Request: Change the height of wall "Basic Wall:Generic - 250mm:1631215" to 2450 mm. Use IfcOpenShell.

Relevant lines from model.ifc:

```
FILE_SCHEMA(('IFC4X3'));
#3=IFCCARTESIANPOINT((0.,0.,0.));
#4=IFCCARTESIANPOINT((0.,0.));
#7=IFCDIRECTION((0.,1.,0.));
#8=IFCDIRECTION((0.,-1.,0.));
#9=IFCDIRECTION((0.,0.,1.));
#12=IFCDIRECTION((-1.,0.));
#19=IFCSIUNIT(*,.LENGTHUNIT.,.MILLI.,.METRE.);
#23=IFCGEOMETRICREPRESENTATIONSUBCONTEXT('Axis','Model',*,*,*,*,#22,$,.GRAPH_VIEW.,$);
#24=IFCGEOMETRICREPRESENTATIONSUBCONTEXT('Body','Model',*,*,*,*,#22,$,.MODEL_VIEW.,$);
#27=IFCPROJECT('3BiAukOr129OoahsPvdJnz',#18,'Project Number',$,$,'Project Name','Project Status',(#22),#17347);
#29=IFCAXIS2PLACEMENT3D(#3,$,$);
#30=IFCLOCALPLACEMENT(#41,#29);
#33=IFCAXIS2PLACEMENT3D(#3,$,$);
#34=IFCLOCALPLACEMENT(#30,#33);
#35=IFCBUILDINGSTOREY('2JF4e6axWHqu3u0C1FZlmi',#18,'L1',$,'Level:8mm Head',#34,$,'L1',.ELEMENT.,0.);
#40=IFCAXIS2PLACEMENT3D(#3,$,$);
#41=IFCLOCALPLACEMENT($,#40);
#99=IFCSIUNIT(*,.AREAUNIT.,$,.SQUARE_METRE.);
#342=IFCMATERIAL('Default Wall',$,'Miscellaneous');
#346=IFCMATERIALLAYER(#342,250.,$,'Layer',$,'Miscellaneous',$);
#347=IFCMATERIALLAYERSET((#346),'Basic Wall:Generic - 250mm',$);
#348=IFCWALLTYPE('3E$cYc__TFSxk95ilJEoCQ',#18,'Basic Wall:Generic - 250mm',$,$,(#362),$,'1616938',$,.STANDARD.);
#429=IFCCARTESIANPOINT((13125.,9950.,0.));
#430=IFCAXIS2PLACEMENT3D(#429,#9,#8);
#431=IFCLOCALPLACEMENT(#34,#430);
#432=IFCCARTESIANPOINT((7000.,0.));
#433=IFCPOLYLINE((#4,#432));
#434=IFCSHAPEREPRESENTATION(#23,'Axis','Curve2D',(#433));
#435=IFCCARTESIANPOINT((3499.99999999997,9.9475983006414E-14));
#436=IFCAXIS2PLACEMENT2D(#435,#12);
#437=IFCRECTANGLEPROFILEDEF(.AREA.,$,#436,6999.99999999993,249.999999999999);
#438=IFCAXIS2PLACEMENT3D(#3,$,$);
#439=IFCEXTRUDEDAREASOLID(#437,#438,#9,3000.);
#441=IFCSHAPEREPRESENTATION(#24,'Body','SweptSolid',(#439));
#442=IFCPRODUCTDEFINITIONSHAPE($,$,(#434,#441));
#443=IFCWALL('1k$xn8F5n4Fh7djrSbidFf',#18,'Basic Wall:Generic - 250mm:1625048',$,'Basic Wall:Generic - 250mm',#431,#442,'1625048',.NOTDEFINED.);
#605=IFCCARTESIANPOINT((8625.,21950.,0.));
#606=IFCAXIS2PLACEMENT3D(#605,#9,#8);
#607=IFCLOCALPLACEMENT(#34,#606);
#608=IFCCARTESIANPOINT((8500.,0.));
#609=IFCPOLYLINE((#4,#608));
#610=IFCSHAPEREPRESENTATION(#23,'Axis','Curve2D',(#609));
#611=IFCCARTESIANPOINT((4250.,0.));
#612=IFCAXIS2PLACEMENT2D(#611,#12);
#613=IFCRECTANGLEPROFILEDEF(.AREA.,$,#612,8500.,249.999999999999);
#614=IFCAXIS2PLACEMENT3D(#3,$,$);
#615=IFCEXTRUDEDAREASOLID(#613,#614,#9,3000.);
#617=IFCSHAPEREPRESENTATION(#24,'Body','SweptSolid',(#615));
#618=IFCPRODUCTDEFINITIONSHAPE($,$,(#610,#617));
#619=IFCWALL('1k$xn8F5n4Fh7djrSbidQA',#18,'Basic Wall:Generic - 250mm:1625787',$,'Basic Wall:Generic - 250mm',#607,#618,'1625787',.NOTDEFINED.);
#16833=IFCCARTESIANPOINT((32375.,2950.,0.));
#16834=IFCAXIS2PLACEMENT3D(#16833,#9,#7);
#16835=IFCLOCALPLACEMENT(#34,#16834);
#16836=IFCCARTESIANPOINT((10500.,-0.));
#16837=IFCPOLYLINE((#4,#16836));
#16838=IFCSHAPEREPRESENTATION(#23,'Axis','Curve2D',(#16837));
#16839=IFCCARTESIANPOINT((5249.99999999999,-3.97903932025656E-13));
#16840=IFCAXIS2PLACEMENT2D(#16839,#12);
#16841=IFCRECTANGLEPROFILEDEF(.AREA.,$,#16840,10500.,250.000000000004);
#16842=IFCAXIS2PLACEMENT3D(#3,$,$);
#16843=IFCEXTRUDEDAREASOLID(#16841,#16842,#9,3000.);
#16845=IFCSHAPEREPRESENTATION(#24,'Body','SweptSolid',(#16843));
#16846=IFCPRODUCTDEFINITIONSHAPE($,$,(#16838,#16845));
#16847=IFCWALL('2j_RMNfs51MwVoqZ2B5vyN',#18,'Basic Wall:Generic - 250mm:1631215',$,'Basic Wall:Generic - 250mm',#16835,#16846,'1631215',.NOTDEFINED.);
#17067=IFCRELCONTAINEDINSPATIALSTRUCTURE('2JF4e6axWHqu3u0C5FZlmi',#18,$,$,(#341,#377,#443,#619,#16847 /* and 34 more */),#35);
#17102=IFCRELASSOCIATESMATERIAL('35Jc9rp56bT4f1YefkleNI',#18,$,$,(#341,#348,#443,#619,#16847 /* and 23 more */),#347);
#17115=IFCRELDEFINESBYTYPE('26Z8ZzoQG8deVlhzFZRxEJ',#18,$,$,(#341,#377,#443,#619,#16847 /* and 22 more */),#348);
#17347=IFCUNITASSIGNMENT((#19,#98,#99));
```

```python
import ifcopenshell
import ifcopenshell.geom
import ifcopenshell.util.representation
import ifcopenshell.util.shape

model = ifcopenshell.open("model.ifc")
settings = ifcopenshell.geom.settings()


def volume(element):
    """Net volume in cubic metres, openings subtracted."""
    shape = ifcopenshell.geom.create_shape(settings, element)
    return ifcopenshell.util.shape.get_volume(shape.geometry)


wall = model.by_id(16847)
before = volume(wall)

body = ifcopenshell.util.representation.get_representation(wall, "Model", "Body")
solid = body.Items[0]
old_height = solid.Depth
solid.Depth = 2450.0
after = volume(wall)

print(f"height {old_height:g} -> {solid.Depth:g}, volume {before:.3f} -> {after:.3f} m3")

model.write("model_edited.ifc")
```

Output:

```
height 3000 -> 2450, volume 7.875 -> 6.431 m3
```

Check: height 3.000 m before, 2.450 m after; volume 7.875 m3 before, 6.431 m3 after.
